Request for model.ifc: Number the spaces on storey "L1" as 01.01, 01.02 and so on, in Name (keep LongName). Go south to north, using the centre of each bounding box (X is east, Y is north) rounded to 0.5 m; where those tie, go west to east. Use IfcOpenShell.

First a look at what the model holds.

```python
import ifcopenshell
import ifcopenshell.util.element
import ifcopenshell.util.placement

model = ifcopenshell.open("model.ifc")
print(model.schema)
storey = next(s for s in model.by_type("IfcBuildingStorey") if s.Name == "L1")
spaces = [e for e in ifcopenshell.util.element.get_decomposition(storey) if e.is_a("IfcSpace")]
for e in sorted(spaces, key=lambda e: e.id()):
    origin = ifcopenshell.util.placement.get_local_placement(e.ObjectPlacement)[:3, 3]
    print(e.id(), e.Name, e.LongName, origin.round(2) + 0.0, sep=" | ")
```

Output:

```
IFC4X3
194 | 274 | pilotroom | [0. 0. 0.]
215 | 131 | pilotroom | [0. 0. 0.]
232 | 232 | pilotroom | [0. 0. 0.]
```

```python
import ifcopenshell
import ifcopenshell.geom
import ifcopenshell.util.element
import ifcopenshell.util.shape

model = ifcopenshell.open("model.ifc")
settings = ifcopenshell.geom.settings()
settings.set("use-world-coords", True)


def centre(element):
    shape = ifcopenshell.geom.create_shape(settings, element)
    return ifcopenshell.util.shape.get_bbox_centroid(shape.geometry)


storey = next(s for s in model.by_type("IfcBuildingStorey") if s.Name == "L1")
spaces = [e for e in ifcopenshell.util.element.get_decomposition(storey) if e.is_a("IfcSpace")]

# Insertion points can sit at a corner or the storey origin, so sort by the geometry (in metres).
centres = {e: centre(e) for e in spaces}
spaces.sort(key=lambda e: (round(centres[e][1] / 0.5), centres[e][0]))

for i, e in enumerate(spaces, start=1):
    number = f"01.{i:02d}"
    e.Name = number
    print(e.id(), number)

model.write("model_edited.ifc")
```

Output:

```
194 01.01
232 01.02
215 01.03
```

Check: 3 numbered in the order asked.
